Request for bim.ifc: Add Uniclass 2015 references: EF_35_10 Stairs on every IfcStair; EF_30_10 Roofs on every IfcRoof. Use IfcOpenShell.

First a look at what the model holds.

```python
import ifcopenshell

model = ifcopenshell.open("bim.ifc")
print(model.schema)
print("classifications:", [c.Name for c in model.by_type("IfcClassification")])
for ifc_class in ("IfcDoor", "IfcRoof", "IfcStair", "IfcWall", "IfcWindow"):
    print(ifc_class, len(model.by_type(ifc_class)))
```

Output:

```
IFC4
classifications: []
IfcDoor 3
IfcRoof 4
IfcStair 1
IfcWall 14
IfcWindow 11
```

```python
import ifcopenshell
import ifcopenshell.api.classification

model = ifcopenshell.open("bim.ifc")

system = ifcopenshell.api.classification.add_classification(model, classification="Uniclass 2015")

codes = {
    "IfcStair": ("EF_35_10", "Stairs"),
    "IfcRoof": ("EF_30_10", "Roofs"),
}
for ifc_class, (code, name) in codes.items():
    products = model.by_type(ifc_class)
    ifcopenshell.api.classification.add_reference(
        model, products=products, classification=system, identification=code, name=name
    )
    print(code, len(products))

model.write("bim_updated.ifc")
```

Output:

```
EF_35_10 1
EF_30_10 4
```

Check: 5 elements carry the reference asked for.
